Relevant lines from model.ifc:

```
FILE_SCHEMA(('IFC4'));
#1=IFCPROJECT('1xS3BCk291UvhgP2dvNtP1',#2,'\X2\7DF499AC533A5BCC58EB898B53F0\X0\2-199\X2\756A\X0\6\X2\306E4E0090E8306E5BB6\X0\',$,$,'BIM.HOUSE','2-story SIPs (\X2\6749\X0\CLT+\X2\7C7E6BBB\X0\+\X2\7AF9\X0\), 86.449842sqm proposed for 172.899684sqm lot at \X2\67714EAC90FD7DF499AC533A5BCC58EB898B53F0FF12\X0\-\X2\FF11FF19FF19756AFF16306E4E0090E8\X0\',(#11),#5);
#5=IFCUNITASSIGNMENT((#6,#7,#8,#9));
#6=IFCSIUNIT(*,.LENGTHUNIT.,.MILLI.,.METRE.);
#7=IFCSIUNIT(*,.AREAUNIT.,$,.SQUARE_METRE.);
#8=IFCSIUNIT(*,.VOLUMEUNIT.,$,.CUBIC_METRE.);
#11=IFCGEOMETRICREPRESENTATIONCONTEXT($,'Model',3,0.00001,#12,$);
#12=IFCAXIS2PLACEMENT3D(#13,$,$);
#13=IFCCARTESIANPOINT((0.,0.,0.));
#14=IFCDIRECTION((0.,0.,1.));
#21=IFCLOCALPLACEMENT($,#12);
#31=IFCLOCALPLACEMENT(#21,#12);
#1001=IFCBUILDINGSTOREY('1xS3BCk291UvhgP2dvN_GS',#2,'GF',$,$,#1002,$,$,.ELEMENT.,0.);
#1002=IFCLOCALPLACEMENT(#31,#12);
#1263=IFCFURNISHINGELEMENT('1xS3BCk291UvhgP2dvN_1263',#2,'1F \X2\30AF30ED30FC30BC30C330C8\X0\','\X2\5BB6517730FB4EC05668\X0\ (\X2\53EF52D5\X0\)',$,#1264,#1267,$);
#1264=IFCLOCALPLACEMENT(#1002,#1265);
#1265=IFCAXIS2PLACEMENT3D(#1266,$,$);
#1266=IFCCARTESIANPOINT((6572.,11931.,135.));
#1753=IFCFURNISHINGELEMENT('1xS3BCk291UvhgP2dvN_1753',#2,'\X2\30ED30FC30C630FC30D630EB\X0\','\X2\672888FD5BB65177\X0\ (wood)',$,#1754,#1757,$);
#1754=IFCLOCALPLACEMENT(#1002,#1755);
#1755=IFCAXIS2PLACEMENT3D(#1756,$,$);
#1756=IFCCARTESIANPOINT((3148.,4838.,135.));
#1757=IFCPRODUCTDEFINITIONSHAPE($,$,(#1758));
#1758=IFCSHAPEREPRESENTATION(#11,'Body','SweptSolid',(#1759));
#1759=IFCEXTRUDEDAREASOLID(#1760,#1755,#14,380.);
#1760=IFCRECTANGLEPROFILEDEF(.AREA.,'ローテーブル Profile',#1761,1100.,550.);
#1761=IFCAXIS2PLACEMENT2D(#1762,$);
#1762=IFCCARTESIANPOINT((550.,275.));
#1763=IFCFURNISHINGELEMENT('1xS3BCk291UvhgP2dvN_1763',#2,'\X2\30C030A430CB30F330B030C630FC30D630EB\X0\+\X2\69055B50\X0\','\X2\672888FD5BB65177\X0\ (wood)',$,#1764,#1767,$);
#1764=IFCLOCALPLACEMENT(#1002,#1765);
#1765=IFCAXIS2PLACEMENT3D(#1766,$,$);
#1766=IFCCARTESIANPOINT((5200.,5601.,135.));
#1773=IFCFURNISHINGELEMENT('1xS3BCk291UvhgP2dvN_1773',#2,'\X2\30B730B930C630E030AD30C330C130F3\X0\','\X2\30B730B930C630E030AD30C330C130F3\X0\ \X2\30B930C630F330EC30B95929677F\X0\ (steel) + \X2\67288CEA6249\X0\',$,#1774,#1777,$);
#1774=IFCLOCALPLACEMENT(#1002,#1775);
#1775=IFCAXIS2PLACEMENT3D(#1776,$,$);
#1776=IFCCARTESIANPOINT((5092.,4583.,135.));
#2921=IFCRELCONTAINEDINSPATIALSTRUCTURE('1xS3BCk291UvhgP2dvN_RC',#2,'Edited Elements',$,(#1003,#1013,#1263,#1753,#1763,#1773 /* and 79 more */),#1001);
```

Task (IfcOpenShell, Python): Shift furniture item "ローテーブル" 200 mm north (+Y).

```python
import ifcopenshell
import ifcopenshell.api.geometry
import ifcopenshell.util.placement

model = ifcopenshell.open("model.ifc")

item = model.by_guid("1xS3BCk291UvhgP2dvN_1753")
matrix = ifcopenshell.util.placement.get_local_placement(item.ObjectPlacement)
matrix[1, 3] += 200.0
ifcopenshell.api.geometry.edit_object_placement(model, product=item, matrix=matrix, is_si=False)

print(ifcopenshell.util.placement.get_local_placement(item.ObjectPlacement).round(3) + 0.0)

model.write("model-out.ifc")
```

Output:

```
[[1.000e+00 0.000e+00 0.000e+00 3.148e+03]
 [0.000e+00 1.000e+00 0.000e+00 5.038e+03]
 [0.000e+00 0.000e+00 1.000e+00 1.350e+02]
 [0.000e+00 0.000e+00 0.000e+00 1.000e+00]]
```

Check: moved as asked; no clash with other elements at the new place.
